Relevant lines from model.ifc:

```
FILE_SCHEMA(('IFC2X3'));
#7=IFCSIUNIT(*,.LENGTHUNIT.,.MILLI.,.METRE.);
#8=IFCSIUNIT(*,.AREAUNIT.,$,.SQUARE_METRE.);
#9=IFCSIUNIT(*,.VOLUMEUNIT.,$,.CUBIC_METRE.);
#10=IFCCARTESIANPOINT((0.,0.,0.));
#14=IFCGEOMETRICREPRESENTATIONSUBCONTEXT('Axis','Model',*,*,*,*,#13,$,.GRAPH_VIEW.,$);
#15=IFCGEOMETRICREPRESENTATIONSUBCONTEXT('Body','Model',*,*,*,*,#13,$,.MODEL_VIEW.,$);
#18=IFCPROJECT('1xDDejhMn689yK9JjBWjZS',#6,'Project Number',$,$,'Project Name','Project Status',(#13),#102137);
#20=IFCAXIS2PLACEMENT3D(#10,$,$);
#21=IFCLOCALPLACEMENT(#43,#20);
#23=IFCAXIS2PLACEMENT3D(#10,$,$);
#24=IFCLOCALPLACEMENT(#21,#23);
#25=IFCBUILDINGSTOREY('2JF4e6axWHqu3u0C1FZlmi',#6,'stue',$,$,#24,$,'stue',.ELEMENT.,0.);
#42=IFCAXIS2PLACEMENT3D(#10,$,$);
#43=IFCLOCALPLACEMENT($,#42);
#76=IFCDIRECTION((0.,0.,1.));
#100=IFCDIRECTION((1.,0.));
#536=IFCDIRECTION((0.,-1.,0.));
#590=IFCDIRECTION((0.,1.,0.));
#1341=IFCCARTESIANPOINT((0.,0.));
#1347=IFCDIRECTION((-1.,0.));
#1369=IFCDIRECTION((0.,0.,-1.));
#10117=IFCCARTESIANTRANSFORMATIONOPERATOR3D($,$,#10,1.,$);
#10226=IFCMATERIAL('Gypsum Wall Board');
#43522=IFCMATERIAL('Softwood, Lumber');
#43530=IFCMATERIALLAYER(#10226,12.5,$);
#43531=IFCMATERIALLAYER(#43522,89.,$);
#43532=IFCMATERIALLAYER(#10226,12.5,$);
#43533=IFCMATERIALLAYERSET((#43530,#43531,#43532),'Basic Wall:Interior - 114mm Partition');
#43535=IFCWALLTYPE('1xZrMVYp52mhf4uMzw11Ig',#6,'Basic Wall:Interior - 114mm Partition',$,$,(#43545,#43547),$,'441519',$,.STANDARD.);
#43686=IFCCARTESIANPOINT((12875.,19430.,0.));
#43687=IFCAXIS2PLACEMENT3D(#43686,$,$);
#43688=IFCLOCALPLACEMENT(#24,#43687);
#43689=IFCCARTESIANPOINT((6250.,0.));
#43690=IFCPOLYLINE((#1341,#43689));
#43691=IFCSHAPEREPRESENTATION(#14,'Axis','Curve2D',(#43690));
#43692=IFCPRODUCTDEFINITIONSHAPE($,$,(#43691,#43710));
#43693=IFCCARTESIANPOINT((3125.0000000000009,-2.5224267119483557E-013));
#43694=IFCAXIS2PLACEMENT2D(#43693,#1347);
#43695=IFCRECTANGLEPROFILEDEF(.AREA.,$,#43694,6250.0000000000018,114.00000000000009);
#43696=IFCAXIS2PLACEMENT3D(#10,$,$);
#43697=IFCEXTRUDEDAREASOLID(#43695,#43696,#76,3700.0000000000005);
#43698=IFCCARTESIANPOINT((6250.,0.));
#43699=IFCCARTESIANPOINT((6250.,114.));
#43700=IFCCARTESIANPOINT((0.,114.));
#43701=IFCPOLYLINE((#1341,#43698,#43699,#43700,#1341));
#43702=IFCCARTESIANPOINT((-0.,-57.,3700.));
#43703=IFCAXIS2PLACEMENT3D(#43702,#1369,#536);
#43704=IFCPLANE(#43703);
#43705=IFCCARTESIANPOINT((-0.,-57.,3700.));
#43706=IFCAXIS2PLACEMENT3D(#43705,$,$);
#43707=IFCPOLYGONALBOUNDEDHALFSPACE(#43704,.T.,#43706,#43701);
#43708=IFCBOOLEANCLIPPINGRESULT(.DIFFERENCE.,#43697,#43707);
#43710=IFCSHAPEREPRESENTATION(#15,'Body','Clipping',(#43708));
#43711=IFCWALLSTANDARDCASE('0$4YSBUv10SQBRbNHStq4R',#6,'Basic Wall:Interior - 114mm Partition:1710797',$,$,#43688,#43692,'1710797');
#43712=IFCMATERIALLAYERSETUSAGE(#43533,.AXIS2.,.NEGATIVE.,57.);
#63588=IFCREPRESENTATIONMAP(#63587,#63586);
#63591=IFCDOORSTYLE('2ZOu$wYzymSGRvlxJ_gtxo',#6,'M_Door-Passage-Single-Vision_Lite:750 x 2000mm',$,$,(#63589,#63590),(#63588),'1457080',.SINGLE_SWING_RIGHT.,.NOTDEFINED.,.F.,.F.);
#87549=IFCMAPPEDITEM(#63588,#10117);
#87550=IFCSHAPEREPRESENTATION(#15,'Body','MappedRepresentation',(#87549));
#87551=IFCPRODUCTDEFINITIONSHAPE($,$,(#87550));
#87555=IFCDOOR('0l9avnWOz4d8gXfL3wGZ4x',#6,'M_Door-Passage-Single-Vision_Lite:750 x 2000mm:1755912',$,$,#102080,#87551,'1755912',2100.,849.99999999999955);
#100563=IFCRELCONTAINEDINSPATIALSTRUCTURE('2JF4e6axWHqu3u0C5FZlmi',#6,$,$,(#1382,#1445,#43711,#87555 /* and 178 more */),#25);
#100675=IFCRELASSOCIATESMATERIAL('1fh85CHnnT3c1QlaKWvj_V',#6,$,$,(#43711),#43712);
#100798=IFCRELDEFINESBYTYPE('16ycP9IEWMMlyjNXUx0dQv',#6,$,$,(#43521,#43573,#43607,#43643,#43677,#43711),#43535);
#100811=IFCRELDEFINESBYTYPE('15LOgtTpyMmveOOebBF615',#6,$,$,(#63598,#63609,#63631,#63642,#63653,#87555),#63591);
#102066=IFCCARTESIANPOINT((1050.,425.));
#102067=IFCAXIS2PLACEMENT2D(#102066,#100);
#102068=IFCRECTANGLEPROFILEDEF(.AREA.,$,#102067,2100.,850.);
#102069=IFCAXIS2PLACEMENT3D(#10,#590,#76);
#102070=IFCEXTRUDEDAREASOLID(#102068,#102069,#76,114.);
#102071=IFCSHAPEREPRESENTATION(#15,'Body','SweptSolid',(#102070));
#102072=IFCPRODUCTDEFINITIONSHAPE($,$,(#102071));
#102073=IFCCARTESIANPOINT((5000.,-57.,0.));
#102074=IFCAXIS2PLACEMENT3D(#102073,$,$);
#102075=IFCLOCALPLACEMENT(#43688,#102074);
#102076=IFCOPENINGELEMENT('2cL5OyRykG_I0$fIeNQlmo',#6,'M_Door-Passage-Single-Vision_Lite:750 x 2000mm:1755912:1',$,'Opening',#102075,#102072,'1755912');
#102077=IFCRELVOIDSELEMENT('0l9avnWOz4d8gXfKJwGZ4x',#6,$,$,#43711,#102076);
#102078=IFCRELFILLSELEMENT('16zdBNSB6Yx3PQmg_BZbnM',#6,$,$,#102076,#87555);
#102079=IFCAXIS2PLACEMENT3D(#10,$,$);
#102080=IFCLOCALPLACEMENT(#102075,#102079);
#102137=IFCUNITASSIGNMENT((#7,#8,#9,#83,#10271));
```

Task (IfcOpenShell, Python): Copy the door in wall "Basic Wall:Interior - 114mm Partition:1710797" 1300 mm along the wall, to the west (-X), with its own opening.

```python
import ifcopenshell
import ifcopenshell.api.feature
import ifcopenshell.api.geometry
import ifcopenshell.api.root
import ifcopenshell.geom
import ifcopenshell.util.element
import ifcopenshell.util.placement
import ifcopenshell.util.shape
import ifcopenshell.util.unit

model = ifcopenshell.open("model.ifc")
unit_scale = ifcopenshell.util.unit.calculate_unit_scale(model)
settings = ifcopenshell.geom.settings()


def volume(element):
    """Net volume in cubic metres, openings subtracted."""
    shape = ifcopenshell.geom.create_shape(settings, element)
    return ifcopenshell.util.shape.get_volume(shape.geometry)


def reuse_history(source, copy):
    """copy_class also copies each property set's owner history, people and application; keep the originals."""
    for rel in copy.IsDefinedBy:
        if rel.is_a("IfcRelDefinesByProperties") and (history := rel.RelatingPropertyDefinition.OwnerHistory):
            rel.RelatingPropertyDefinition.OwnerHistory = source.OwnerHistory
            ifcopenshell.util.element.remove_deep2(model, history)


door = model.by_id(87555)
opening = door.FillsVoids[0].RelatingOpeningElement
wall = opening.VoidsElements[0].RelatingBuildingElement
before = volume(wall)
shift = ifcopenshell.util.placement.get_local_placement(wall.ObjectPlacement)[:3, 0] * -1.3 / unit_scale

# copy_class copies the void relationship, type, container and properties, but no geometry.
new_opening = ifcopenshell.api.root.copy_class(model, product=opening)
new_opening.Representation = ifcopenshell.util.element.copy_deep(
    model, opening.Representation, exclude=["IfcGeometricRepresentationContext", "IfcRepresentationMap"]
)
new_opening.Name = "M_Door-Passage-Single-Vision_Lite:750 x 2000mm"
new_opening.Tag = None
new_door = ifcopenshell.api.root.copy_class(model, product=door)
new_door.Representation = ifcopenshell.util.element.copy_deep(
    model, door.Representation, exclude=["IfcGeometricRepresentationContext", "IfcRepresentationMap"]
)
new_door.Name = "M_Door-Passage-Single-Vision_Lite:750 x 2000mm"
new_door.Tag = None
reuse_history(door, new_door)
fills = ifcopenshell.api.feature.add_filling(model, opening=new_opening, element=new_door)
fills.OwnerHistory = new_door.OwnerHistory  # required in IFC2X3

for old, new in ((opening, new_opening), (door, new_door)):
    matrix = ifcopenshell.util.placement.get_local_placement(old.ObjectPlacement)
    matrix[:3, 3] += shift
    ifcopenshell.api.geometry.edit_object_placement(model, product=new, matrix=matrix, is_si=False)

after = volume(wall)

print(f"wall volume {before:.3f} -> {after:.3f} m3")

model.write("model_rev.ifc")
```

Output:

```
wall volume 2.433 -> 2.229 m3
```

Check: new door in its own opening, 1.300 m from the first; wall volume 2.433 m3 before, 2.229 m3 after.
